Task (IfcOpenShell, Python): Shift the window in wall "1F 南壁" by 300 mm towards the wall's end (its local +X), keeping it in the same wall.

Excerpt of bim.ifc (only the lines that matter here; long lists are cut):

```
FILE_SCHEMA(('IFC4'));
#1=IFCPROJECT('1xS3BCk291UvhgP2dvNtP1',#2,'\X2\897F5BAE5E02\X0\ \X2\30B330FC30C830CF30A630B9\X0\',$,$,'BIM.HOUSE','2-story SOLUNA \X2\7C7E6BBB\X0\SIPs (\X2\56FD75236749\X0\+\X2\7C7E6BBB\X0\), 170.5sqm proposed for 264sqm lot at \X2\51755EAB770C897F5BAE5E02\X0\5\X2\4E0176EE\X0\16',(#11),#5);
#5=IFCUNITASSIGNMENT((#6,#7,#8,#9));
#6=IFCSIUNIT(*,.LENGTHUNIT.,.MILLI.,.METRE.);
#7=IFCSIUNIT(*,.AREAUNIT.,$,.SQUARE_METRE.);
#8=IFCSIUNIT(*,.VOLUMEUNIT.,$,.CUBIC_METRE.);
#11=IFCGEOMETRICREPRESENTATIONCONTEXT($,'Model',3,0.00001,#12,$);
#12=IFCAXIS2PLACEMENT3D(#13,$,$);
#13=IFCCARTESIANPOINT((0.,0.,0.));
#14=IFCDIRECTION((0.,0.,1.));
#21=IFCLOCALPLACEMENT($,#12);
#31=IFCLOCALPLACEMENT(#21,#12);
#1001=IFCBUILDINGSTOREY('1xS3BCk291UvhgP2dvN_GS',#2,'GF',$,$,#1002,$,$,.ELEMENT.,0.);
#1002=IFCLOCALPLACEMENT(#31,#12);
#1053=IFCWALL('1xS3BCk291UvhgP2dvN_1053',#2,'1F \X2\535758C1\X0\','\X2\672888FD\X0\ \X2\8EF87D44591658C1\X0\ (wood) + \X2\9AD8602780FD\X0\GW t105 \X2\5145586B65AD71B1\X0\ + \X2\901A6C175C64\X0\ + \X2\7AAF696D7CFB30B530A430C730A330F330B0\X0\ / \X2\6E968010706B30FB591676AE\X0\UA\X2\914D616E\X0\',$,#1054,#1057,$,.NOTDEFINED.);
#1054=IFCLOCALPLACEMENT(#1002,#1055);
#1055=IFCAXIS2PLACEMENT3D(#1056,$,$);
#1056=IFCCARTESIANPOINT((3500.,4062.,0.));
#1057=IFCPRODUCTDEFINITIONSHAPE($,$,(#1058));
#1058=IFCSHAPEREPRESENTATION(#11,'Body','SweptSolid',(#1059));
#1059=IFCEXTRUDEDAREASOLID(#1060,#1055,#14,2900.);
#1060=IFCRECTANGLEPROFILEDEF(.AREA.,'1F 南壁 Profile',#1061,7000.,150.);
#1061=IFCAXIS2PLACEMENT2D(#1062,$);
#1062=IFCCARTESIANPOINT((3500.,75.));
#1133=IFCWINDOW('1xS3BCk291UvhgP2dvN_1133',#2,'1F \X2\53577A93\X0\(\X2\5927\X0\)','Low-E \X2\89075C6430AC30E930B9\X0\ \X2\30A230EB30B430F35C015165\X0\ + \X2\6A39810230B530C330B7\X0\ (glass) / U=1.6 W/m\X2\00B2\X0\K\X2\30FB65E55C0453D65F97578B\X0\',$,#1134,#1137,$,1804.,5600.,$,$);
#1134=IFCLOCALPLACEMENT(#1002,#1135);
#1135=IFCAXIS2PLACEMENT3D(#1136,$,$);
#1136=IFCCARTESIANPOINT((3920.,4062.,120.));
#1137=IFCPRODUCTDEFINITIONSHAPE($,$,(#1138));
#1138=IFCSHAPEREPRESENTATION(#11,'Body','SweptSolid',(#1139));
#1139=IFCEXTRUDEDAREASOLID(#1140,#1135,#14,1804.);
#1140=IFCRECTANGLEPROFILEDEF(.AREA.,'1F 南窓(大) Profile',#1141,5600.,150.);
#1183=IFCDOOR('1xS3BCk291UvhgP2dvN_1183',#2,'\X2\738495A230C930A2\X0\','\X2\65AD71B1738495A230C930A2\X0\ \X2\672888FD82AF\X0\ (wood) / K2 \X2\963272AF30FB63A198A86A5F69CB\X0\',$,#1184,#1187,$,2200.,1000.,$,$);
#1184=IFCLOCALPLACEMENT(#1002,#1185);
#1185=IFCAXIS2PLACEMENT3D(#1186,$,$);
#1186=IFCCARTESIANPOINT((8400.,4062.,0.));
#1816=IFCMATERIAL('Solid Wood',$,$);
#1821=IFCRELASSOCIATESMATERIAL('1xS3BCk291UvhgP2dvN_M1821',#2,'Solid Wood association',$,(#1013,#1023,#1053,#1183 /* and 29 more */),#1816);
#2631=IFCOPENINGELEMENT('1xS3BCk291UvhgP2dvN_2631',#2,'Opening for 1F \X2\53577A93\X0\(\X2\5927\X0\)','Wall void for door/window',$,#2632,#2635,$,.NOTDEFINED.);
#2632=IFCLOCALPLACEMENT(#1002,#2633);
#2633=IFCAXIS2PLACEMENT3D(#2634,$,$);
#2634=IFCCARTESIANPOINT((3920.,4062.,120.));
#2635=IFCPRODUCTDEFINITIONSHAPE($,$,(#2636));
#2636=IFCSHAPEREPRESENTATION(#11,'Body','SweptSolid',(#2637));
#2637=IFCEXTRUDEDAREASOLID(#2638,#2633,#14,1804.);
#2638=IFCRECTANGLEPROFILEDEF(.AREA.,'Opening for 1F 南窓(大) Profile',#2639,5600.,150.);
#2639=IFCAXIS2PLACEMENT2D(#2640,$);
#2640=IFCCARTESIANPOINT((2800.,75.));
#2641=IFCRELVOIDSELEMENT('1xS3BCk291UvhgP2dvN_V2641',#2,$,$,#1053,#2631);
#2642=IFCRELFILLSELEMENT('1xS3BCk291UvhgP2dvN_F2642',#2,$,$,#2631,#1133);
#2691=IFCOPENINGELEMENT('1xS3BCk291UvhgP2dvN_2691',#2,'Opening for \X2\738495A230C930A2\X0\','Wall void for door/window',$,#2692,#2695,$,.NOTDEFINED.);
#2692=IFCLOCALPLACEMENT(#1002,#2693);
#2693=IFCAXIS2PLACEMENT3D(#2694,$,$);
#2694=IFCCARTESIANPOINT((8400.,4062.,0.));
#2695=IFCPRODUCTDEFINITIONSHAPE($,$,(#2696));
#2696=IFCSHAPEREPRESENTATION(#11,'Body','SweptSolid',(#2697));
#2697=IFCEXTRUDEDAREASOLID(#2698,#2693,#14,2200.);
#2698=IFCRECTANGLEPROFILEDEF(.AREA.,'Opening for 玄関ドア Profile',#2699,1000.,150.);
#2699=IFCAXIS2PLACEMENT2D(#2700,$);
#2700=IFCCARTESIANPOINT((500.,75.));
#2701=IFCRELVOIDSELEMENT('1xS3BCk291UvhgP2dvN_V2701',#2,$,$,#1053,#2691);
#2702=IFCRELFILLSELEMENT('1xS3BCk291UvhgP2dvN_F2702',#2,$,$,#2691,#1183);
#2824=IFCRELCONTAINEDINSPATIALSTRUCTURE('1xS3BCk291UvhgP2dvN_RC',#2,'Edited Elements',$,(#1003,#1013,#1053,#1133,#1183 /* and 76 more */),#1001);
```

```python
import ifcopenshell
import ifcopenshell.api.geometry
import ifcopenshell.util.placement
import ifcopenshell.util.unit

model = ifcopenshell.open("bim.ifc")
unit_scale = ifcopenshell.util.unit.calculate_unit_scale(model)

window = model.by_id(1133)
opening = window.FillsVoids[0].RelatingOpeningElement
wall = opening.VoidsElements[0].RelatingBuildingElement

wall_matrix = ifcopenshell.util.placement.get_local_placement(wall.ObjectPlacement)
shift = wall_matrix[:3, 0] * 0.3 / unit_scale
before = ifcopenshell.util.placement.get_local_placement(window.ObjectPlacement)[:3, 3].copy()

# The window is not placed relative to its opening, so move both.
for product in (opening, window):
    matrix = ifcopenshell.util.placement.get_local_placement(product.ObjectPlacement)
    matrix[:3, 3] += shift
    ifcopenshell.api.geometry.edit_object_placement(model, product=product, matrix=matrix, is_si=False)

after = ifcopenshell.util.placement.get_local_placement(window.ObjectPlacement)[:3, 3]
print("window moved by", (after - before).round(3) + 0.0)

model.write("bim_rev.ifc")
```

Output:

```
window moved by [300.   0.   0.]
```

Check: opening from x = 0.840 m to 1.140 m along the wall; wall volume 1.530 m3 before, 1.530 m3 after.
